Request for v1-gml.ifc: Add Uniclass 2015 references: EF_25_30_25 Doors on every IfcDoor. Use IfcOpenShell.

First a look at what the model holds.

```python
import ifcopenshell

model = ifcopenshell.open("v1-gml.ifc")
print(model.schema)
print("classifications:", [c.Name for c in model.by_type("IfcClassification")])
for ifc_class in ("IfcDoor", "IfcRoof", "IfcStair", "IfcWall", "IfcWindow"):
    print(ifc_class, len(model.by_type(ifc_class)))
```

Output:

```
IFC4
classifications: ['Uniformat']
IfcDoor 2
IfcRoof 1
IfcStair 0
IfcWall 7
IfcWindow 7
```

```python
import ifcopenshell
import ifcopenshell.api.classification

model = ifcopenshell.open("v1-gml.ifc")

system = ifcopenshell.api.classification.add_classification(model, classification="Uniclass 2015")

codes = {
    "IfcDoor": ("EF_25_30_25", "Doors"),
}
for ifc_class, (code, name) in codes.items():
    products = model.by_type(ifc_class)
    ifcopenshell.api.classification.add_reference(
        model, products=products, classification=system, identification=code, name=name
    )
    print(code, len(products))

model.write("v1-gml_rev.ifc")
```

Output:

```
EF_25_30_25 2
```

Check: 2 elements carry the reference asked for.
